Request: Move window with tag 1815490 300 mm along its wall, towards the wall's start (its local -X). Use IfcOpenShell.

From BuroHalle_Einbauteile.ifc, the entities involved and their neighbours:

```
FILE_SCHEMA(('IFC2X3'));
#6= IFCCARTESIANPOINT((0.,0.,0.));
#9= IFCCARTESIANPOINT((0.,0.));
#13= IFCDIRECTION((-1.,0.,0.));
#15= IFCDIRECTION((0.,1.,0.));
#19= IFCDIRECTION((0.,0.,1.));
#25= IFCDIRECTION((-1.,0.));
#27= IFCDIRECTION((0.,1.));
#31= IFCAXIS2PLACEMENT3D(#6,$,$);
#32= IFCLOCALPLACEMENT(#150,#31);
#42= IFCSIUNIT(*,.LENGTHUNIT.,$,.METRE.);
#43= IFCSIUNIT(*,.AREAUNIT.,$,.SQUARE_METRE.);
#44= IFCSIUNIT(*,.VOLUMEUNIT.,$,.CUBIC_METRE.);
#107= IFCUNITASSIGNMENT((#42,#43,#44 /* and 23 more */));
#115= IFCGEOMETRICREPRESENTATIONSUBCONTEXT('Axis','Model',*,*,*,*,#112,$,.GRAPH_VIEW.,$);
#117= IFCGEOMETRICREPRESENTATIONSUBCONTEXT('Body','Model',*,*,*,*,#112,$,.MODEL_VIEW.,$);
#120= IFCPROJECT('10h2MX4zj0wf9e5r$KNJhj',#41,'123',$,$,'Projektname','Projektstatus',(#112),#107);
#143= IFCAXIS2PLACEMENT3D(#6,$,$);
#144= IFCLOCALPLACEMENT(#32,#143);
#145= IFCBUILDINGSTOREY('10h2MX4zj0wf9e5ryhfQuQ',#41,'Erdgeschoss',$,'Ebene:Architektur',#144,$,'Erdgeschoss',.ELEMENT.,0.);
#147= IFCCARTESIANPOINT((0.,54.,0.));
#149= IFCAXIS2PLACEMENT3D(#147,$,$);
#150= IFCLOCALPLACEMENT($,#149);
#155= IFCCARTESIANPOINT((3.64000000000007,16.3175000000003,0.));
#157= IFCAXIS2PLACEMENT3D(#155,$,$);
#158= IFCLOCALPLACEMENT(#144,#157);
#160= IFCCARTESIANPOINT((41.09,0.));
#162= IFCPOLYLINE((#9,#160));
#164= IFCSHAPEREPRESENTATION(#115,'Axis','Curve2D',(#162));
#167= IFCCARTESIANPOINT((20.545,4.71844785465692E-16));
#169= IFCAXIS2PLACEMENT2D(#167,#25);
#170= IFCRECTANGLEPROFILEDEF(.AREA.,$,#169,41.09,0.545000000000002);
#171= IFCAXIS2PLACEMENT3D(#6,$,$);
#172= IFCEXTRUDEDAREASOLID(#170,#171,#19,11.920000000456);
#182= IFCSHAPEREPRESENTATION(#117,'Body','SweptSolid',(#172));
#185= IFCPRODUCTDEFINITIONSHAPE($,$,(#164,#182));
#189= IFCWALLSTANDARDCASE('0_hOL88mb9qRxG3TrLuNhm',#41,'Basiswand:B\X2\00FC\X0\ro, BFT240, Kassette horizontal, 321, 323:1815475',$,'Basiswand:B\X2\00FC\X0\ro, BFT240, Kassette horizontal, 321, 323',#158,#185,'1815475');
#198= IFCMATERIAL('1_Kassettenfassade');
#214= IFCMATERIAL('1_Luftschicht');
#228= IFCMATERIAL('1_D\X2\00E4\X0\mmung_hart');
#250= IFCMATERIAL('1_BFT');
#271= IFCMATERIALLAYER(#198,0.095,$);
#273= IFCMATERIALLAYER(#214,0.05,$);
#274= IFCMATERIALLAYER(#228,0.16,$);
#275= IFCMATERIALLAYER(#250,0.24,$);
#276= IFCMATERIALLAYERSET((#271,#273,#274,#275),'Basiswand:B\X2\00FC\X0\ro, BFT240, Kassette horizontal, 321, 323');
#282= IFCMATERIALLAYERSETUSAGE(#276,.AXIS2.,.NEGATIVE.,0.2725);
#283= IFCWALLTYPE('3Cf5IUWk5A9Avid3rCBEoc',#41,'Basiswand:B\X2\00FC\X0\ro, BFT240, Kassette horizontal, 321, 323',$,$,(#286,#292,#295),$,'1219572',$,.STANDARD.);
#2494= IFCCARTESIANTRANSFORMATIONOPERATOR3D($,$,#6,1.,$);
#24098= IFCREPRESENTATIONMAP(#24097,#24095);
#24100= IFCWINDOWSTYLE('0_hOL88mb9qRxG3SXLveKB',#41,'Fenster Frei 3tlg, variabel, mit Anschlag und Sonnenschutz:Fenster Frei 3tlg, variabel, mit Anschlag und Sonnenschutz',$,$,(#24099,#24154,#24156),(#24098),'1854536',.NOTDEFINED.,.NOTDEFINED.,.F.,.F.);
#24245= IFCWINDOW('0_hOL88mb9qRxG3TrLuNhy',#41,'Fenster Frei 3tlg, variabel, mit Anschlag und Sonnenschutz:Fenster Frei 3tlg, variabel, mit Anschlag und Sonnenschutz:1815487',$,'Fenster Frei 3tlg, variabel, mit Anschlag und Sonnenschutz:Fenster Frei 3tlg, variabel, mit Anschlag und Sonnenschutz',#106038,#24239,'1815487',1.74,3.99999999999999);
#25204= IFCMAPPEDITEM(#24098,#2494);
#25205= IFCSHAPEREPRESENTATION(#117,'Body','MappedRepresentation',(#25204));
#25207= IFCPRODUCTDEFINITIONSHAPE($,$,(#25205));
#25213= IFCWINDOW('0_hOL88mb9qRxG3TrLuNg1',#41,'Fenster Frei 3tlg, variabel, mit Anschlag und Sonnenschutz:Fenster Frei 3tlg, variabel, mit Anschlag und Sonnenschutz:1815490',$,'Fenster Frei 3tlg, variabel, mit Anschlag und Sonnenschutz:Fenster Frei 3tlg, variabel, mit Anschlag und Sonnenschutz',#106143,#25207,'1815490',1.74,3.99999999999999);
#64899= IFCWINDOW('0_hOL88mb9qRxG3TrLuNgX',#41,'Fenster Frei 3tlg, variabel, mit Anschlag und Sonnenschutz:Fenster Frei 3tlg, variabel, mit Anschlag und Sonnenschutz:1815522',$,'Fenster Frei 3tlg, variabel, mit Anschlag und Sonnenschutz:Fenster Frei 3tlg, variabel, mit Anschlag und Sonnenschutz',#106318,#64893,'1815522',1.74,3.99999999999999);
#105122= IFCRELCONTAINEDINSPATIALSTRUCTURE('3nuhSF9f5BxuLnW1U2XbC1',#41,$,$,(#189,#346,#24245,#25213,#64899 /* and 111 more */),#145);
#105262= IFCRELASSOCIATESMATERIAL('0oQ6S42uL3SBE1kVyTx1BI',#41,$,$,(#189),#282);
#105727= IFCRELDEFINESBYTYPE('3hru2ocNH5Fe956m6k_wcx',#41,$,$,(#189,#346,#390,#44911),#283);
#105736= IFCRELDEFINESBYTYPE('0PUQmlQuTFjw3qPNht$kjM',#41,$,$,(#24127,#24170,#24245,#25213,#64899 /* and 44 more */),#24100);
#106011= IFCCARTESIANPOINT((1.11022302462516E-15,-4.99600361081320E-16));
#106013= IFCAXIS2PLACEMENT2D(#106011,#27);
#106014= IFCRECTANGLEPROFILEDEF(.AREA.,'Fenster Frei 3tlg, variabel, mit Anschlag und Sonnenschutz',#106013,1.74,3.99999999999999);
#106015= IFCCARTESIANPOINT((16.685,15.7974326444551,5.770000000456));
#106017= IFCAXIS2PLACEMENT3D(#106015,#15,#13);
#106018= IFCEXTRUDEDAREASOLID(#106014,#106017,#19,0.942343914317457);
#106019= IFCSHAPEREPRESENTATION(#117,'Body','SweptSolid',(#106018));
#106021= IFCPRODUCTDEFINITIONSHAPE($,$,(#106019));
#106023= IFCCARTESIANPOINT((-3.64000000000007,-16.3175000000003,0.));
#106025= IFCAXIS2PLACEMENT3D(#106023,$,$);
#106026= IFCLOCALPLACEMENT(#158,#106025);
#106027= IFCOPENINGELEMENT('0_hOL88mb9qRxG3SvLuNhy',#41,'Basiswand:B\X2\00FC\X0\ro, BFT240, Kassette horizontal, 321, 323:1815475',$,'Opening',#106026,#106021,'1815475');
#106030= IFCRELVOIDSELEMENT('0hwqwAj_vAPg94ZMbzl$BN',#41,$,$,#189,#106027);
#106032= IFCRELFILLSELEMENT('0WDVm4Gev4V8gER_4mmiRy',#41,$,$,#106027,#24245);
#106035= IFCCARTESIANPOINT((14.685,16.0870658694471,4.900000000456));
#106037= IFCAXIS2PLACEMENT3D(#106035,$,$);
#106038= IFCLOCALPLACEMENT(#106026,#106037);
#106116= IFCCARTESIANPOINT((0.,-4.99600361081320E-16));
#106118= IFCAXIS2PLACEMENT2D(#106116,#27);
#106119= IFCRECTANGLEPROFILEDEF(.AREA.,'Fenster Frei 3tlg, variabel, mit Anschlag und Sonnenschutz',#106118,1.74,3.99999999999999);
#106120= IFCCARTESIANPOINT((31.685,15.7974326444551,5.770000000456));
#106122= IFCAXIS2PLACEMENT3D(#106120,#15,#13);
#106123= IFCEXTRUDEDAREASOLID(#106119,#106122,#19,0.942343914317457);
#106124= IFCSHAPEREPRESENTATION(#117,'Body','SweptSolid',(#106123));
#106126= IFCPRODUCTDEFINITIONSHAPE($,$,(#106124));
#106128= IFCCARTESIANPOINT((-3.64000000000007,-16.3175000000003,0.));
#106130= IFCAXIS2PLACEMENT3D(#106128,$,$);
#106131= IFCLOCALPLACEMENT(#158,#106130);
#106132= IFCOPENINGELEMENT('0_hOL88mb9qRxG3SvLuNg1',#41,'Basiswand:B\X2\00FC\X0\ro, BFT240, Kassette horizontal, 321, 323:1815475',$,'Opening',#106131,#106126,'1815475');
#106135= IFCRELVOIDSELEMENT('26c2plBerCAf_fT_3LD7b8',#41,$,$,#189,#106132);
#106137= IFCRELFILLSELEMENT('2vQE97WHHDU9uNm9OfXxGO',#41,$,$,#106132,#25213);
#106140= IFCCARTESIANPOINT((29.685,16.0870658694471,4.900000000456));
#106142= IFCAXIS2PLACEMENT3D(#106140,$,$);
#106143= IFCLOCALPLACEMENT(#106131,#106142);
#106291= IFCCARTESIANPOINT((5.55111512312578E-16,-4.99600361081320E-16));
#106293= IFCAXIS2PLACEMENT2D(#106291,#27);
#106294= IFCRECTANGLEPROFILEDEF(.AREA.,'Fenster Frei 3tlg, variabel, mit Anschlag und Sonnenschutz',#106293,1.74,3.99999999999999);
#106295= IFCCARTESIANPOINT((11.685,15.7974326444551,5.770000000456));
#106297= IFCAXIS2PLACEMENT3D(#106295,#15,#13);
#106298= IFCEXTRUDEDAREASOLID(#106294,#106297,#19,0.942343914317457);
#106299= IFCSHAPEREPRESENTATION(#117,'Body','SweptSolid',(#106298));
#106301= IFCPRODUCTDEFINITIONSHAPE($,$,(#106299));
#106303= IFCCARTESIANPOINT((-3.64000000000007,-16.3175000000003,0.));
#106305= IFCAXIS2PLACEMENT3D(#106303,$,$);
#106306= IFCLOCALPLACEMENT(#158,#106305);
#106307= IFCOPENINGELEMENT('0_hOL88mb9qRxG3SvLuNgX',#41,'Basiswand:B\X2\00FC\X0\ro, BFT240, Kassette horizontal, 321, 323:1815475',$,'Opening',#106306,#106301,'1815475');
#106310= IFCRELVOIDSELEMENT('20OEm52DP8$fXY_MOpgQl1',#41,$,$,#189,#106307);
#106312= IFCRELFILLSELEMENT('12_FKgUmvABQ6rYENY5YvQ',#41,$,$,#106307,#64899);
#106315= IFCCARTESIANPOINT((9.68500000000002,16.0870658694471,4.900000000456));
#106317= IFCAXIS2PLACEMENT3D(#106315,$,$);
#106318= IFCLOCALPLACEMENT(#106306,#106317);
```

```python
import ifcopenshell
import ifcopenshell.api.geometry
import ifcopenshell.util.placement
import ifcopenshell.util.unit

model = ifcopenshell.open("BuroHalle_Einbauteile.ifc")
unit_scale = ifcopenshell.util.unit.calculate_unit_scale(model)

window = model.by_guid("0_hOL88mb9qRxG3TrLuNg1")
opening = window.FillsVoids[0].RelatingOpeningElement
wall = opening.VoidsElements[0].RelatingBuildingElement

wall_matrix = ifcopenshell.util.placement.get_local_placement(wall.ObjectPlacement)
shift = wall_matrix[:3, 0] * -0.3 / unit_scale
before = ifcopenshell.util.placement.get_local_placement(window.ObjectPlacement)[:3, 3].copy()

# The window is placed relative to its opening, so it follows when the opening moves.
matrix = ifcopenshell.util.placement.get_local_placement(opening.ObjectPlacement)
matrix[:3, 3] += shift
ifcopenshell.api.geometry.edit_object_placement(
    model, product=opening, matrix=matrix, is_si=False, should_transform_children=True
)

after = ifcopenshell.util.placement.get_local_placement(window.ObjectPlacement)[:3, 3]
print("window moved by", (after - before).round(3) + 0.0)

model.write("BuroHalle_Einbauteile_updated.ifc")
```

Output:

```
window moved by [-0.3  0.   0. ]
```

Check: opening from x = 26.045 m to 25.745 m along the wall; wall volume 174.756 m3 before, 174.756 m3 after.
